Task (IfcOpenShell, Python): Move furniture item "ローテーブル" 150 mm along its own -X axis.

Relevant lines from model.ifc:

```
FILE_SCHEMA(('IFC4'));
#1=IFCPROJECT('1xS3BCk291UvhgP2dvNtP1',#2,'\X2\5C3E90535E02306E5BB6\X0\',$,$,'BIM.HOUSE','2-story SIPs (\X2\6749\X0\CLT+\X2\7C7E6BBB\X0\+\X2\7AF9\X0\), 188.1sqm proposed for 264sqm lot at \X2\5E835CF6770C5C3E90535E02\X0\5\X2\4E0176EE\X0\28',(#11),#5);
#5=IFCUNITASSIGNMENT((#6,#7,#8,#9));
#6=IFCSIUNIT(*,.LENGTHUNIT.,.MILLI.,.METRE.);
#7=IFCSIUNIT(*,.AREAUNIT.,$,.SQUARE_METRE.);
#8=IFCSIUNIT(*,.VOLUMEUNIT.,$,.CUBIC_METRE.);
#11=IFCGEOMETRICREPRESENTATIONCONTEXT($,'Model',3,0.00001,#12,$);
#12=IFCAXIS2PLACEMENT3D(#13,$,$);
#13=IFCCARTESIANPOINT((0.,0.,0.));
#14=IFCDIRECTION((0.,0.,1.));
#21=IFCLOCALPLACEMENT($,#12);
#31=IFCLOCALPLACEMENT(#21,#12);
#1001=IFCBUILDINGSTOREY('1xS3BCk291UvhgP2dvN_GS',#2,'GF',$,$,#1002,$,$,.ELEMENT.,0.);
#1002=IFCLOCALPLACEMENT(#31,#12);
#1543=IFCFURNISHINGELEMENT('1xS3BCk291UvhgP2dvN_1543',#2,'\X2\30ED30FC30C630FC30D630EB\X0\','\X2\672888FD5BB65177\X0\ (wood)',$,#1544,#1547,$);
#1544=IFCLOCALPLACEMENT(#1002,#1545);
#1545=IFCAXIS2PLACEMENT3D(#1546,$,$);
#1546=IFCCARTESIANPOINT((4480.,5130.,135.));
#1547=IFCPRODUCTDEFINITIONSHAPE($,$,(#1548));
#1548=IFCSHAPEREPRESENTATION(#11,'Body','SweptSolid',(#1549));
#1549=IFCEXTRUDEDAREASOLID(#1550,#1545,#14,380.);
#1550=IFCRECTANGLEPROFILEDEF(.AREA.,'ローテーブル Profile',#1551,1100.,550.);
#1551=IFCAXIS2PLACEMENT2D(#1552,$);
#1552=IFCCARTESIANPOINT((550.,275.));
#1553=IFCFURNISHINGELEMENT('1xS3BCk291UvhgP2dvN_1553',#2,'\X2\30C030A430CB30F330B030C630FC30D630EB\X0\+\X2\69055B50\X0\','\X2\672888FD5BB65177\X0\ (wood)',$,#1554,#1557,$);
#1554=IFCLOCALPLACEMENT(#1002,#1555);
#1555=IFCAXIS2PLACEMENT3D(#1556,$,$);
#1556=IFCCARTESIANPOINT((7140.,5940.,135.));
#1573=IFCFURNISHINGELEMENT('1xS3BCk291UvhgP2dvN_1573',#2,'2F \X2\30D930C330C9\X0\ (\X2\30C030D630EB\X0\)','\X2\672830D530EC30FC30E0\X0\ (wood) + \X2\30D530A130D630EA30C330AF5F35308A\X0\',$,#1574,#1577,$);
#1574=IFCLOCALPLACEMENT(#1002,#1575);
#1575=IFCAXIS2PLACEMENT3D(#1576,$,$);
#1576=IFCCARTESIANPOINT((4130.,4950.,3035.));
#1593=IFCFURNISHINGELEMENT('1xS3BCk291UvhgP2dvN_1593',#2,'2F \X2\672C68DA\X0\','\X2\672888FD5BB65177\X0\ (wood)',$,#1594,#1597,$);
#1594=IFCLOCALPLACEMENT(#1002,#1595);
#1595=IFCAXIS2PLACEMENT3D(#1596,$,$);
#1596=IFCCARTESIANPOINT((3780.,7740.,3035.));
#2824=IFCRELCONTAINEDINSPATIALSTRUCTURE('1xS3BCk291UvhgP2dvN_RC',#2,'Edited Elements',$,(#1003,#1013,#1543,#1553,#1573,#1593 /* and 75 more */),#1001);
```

```python
import ifcopenshell
import ifcopenshell.api.geometry
import ifcopenshell.util.placement

model = ifcopenshell.open("model.ifc")

item = model.by_guid("1xS3BCk291UvhgP2dvN_1543")
matrix = ifcopenshell.util.placement.get_local_placement(item.ObjectPlacement)
matrix[:3, 3] -= matrix[:3, 0] * 150.0
ifcopenshell.api.geometry.edit_object_placement(model, product=item, matrix=matrix, is_si=False)

print(ifcopenshell.util.placement.get_local_placement(item.ObjectPlacement).round(3) + 0.0)

model.write("model_v2.ifc")
```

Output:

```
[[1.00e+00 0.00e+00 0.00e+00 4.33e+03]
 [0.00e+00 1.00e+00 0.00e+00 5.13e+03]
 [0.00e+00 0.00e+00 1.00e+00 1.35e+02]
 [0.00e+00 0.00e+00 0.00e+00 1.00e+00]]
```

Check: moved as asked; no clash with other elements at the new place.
